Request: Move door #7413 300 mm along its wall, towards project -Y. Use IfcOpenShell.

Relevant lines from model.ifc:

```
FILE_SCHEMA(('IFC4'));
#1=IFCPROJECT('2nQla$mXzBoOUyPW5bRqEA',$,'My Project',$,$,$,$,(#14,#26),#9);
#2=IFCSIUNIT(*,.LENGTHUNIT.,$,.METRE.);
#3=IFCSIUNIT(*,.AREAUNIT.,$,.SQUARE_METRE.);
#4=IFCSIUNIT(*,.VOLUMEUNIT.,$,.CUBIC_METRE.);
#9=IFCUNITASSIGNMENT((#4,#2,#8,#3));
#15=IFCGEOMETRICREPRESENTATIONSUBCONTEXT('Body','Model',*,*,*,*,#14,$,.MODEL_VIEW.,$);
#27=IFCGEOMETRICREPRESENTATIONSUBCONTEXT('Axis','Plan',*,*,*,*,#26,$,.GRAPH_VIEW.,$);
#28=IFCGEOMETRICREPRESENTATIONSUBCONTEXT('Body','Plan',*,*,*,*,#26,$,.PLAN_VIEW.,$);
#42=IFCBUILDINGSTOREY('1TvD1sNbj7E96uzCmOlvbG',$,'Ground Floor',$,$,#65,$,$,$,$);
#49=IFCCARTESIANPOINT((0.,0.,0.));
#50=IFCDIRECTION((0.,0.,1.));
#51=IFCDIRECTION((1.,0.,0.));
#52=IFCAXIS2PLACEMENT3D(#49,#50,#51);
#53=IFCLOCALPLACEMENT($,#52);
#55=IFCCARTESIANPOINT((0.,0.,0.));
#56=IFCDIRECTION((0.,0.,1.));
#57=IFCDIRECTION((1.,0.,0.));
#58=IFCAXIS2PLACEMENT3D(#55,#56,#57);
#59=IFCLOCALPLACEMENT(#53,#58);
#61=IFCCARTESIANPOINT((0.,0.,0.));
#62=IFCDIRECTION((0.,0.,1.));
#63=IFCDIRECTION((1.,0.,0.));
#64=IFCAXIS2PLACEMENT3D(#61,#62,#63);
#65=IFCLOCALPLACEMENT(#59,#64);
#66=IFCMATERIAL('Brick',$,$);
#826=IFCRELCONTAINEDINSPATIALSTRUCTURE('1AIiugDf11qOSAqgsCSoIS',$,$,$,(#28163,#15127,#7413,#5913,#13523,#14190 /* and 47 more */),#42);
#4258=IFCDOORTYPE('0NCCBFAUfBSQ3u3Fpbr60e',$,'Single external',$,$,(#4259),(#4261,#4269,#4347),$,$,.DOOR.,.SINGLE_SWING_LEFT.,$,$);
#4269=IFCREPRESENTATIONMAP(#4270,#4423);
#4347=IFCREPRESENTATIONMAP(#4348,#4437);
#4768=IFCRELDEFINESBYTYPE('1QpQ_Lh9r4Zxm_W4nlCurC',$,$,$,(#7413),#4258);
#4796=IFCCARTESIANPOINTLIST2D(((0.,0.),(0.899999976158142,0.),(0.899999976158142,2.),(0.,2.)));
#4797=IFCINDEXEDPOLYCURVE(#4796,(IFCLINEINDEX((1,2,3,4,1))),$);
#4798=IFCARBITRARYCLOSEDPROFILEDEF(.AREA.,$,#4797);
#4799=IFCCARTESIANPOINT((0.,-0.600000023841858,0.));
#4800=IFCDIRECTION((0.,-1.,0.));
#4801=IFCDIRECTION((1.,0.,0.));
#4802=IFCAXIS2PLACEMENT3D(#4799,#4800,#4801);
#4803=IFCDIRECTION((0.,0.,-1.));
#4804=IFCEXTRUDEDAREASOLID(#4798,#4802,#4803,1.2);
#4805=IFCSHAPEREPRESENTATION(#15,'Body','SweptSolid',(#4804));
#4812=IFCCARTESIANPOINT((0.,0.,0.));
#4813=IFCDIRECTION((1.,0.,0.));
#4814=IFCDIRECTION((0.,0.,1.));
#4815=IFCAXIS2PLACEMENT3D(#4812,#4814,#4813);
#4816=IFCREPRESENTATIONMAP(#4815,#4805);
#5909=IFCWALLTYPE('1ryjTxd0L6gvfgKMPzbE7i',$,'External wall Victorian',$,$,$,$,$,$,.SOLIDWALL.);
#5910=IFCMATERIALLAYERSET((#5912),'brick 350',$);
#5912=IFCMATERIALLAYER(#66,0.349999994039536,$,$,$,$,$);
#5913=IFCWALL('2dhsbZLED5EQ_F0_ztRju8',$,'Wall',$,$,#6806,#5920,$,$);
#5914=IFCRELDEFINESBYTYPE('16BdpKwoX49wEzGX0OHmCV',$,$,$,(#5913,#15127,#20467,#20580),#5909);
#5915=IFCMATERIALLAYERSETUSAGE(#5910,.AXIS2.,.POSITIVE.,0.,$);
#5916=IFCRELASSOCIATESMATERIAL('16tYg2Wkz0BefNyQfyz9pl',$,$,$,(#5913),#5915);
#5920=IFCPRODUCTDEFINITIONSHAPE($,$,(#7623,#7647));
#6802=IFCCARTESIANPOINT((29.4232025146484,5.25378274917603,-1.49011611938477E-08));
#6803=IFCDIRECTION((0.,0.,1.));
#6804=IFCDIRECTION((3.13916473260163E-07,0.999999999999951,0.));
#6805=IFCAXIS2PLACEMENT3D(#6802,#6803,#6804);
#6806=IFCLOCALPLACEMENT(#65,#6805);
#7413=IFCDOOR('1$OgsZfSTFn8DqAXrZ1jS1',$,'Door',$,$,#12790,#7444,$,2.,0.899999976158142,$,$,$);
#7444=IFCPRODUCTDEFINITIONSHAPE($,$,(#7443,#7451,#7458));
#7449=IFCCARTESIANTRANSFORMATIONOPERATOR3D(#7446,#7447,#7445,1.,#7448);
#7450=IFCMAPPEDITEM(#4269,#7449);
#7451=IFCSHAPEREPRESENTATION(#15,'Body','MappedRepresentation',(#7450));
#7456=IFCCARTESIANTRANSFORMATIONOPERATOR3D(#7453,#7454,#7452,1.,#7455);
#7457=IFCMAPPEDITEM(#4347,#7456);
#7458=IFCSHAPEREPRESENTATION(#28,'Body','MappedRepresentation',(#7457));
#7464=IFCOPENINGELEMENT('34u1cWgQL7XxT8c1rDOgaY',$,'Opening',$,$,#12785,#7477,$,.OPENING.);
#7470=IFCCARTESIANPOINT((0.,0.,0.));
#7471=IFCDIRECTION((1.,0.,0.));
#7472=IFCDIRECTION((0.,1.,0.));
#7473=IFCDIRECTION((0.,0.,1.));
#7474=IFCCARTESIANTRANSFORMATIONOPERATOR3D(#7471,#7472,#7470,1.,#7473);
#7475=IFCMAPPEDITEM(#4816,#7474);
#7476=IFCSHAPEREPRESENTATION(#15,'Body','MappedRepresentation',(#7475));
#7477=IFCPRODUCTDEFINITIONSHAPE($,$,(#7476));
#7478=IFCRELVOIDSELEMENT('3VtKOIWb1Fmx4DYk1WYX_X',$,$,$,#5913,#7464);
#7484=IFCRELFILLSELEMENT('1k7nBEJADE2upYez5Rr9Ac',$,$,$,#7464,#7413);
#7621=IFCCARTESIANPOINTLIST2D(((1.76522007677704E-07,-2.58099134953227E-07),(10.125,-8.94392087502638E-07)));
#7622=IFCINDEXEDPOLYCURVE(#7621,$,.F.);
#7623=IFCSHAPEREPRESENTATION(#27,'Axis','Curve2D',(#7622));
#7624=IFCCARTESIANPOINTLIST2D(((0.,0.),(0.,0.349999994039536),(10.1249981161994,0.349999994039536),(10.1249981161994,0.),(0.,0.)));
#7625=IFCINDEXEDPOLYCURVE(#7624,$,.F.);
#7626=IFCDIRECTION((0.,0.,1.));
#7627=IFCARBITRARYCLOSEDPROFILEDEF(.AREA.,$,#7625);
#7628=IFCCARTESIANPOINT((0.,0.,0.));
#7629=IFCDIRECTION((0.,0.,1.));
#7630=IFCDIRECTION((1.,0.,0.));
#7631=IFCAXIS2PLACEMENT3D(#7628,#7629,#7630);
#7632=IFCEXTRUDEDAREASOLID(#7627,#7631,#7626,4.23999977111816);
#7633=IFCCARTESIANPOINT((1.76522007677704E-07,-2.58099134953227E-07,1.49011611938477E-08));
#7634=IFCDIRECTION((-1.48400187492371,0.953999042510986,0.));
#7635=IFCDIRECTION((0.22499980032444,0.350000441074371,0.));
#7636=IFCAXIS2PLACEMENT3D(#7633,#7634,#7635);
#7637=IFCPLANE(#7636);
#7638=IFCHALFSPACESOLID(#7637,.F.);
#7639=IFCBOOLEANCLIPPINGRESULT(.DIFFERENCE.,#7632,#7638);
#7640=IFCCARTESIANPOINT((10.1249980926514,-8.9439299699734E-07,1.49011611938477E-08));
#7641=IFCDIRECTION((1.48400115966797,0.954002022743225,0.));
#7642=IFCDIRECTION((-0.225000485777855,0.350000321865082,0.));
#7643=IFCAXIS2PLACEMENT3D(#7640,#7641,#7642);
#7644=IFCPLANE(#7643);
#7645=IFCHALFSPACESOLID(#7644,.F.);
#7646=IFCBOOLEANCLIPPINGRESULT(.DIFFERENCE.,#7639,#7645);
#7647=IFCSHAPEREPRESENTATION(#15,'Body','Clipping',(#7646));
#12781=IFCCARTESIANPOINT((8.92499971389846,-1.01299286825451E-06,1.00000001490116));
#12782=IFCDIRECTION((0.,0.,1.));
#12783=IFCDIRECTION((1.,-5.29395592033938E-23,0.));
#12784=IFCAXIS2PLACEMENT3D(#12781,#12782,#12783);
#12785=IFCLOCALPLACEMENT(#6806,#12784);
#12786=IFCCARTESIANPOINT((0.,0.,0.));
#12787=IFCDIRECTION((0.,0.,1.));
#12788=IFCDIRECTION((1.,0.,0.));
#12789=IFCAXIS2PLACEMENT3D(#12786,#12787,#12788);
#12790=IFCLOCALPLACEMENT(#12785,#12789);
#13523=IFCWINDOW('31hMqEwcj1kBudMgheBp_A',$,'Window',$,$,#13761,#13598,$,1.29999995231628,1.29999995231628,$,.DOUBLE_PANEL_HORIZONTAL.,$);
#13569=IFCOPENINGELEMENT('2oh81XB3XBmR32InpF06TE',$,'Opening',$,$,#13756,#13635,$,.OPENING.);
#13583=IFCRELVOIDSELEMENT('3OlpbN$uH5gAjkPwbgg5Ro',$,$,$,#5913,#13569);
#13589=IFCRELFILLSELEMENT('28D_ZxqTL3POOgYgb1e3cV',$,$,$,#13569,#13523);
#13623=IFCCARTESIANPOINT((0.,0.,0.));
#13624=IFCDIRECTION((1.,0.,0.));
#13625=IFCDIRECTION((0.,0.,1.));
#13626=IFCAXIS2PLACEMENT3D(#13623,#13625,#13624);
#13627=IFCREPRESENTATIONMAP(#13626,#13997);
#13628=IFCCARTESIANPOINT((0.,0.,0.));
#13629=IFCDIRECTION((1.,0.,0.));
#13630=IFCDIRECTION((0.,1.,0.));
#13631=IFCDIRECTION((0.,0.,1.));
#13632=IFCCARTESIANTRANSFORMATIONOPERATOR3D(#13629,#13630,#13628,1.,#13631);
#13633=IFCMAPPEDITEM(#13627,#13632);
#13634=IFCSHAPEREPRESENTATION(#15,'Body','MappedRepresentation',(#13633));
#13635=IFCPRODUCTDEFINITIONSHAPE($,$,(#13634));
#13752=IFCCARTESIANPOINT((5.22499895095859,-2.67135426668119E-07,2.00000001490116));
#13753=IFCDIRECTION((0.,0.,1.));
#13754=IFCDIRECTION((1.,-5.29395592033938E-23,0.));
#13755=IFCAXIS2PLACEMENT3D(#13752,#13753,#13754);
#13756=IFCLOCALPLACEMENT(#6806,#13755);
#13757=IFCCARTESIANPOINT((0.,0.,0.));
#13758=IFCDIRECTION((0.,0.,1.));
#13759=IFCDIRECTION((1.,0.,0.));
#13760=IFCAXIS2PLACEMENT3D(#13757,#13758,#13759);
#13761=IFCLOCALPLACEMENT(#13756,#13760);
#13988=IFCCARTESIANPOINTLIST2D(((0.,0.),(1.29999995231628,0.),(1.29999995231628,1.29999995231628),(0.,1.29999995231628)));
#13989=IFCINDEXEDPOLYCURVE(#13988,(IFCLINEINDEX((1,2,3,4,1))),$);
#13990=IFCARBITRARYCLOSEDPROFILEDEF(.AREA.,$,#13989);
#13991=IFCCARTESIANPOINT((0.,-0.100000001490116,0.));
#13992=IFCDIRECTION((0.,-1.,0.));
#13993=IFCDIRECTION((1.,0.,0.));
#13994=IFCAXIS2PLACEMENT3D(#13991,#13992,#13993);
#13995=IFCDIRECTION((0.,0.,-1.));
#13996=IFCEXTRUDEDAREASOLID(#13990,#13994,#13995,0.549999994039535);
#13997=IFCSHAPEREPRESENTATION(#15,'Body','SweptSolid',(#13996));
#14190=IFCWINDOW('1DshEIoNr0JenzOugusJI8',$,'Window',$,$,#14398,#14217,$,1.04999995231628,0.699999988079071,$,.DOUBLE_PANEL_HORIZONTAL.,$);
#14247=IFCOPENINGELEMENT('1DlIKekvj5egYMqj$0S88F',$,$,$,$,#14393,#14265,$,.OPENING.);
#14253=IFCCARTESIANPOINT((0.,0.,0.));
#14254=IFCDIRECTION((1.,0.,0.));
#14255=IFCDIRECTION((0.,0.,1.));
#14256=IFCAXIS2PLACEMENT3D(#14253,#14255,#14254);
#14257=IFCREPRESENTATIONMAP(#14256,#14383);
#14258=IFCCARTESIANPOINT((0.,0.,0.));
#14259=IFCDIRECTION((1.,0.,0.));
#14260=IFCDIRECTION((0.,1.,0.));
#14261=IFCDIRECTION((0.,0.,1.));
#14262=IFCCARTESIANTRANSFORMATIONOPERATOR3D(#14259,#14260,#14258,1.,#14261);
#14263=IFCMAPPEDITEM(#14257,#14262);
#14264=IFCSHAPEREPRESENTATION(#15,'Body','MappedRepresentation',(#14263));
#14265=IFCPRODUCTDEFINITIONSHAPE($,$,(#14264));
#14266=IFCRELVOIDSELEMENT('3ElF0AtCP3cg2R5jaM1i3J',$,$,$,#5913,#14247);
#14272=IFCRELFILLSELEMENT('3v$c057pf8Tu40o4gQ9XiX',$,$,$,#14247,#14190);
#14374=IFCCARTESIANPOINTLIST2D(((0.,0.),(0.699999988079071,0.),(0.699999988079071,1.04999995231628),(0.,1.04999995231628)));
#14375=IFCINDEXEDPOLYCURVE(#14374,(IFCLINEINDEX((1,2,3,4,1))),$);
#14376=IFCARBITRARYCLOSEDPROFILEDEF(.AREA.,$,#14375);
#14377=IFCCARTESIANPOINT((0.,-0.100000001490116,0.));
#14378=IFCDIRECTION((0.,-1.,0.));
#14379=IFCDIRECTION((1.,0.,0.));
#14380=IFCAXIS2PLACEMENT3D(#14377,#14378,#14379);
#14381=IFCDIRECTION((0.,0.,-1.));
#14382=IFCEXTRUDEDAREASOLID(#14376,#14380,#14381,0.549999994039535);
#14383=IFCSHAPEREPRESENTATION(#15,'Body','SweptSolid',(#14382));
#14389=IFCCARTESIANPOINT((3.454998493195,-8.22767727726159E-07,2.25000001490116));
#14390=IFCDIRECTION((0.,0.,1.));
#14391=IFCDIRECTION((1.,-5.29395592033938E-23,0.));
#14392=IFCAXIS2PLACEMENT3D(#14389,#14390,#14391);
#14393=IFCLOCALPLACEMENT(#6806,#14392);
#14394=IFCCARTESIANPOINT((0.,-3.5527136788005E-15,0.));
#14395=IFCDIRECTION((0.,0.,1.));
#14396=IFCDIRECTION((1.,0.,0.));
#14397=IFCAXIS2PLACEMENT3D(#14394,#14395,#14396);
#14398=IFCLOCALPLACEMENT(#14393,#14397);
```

```python
import ifcopenshell
import ifcopenshell.api.geometry
import ifcopenshell.util.placement
import ifcopenshell.util.unit

model = ifcopenshell.open("model.ifc")
unit_scale = ifcopenshell.util.unit.calculate_unit_scale(model)

door = model.by_guid("1$OgsZfSTFn8DqAXrZ1jS1")
opening = door.FillsVoids[0].RelatingOpeningElement
wall = opening.VoidsElements[0].RelatingBuildingElement

wall_matrix = ifcopenshell.util.placement.get_local_placement(wall.ObjectPlacement)
shift = wall_matrix[:3, 0] * -0.3 / unit_scale
before = ifcopenshell.util.placement.get_local_placement(door.ObjectPlacement)[:3, 3].copy()

# The door is placed relative to its opening, so it follows when the opening moves.
matrix = ifcopenshell.util.placement.get_local_placement(opening.ObjectPlacement)
matrix[:3, 3] += shift
ifcopenshell.api.geometry.edit_object_placement(
    model, product=opening, matrix=matrix, is_si=False, should_transform_children=True
)

after = ifcopenshell.util.placement.get_local_placement(door.ObjectPlacement)[:3, 3]
print("door moved by", (after - before).round(3) + 0.0)

model.write("model_edited.ifc")
```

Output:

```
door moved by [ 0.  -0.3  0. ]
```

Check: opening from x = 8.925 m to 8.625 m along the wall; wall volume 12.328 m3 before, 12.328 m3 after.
